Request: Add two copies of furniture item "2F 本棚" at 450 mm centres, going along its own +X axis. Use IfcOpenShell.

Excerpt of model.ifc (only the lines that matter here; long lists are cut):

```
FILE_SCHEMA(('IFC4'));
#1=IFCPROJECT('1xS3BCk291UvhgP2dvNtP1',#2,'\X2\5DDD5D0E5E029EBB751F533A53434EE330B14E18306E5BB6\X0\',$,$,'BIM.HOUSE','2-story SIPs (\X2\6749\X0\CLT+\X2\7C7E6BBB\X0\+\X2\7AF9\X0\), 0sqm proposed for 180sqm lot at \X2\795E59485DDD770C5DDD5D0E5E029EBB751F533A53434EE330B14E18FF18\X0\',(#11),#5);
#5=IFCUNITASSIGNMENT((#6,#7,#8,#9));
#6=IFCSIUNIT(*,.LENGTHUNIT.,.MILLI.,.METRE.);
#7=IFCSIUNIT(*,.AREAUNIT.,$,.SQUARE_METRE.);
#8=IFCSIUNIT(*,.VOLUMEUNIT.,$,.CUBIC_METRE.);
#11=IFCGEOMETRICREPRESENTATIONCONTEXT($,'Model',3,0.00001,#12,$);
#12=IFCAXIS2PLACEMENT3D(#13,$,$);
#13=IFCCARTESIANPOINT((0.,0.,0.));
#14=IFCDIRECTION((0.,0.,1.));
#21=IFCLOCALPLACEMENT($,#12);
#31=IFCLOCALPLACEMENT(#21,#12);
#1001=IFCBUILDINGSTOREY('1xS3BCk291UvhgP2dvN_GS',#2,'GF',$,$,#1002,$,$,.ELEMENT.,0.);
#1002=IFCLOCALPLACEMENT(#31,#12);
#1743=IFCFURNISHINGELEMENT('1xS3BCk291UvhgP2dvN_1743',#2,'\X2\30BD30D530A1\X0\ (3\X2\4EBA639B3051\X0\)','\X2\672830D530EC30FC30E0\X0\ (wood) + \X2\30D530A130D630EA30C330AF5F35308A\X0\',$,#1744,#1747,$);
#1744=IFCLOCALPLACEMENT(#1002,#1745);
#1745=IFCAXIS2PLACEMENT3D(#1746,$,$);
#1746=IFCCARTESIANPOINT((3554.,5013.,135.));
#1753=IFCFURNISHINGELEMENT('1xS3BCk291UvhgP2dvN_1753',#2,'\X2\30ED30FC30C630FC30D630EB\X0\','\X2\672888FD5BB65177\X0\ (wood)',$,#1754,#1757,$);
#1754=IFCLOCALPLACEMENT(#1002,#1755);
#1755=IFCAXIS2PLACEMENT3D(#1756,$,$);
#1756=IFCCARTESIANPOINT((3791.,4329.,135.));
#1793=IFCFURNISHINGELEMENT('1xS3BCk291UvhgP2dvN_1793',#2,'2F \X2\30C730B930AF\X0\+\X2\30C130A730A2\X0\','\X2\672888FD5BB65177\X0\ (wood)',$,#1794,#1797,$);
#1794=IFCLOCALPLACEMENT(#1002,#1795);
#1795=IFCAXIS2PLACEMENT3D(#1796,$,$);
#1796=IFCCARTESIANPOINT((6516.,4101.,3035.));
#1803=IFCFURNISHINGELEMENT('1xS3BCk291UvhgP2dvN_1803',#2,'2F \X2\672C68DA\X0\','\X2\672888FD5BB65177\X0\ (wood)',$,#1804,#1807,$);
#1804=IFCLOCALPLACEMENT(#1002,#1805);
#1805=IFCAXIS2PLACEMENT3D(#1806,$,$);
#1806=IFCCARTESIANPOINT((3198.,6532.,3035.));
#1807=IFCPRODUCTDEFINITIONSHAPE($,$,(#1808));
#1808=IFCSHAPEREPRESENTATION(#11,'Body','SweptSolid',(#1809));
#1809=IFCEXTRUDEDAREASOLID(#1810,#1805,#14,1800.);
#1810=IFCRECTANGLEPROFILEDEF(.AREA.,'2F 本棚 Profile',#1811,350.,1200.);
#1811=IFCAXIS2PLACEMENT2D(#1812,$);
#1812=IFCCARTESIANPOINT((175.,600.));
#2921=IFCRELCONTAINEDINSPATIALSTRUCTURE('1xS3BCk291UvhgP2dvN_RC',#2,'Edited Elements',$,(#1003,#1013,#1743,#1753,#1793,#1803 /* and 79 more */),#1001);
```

```python
import ifcopenshell
import ifcopenshell.api.geometry
import ifcopenshell.api.root
import ifcopenshell.util.element
import ifcopenshell.util.placement
import ifcopenshell.util.unit

model = ifcopenshell.open("model.ifc")
unit_scale = ifcopenshell.util.unit.calculate_unit_scale(model)


def reuse_history(source, copy):
    """copy_class also copies each property set's owner history, people and application; keep the originals."""
    for rel in copy.IsDefinedBy:
        if rel.is_a("IfcRelDefinesByProperties") and (history := rel.RelatingPropertyDefinition.OwnerHistory):
            rel.RelatingPropertyDefinition.OwnerHistory = source.OwnerHistory
            ifcopenshell.util.element.remove_deep2(model, history)


source = model.by_guid("1xS3BCk291UvhgP2dvN_1803")
base = ifcopenshell.util.placement.get_local_placement(source.ObjectPlacement)
step = base[:3, 0] * 0.45 / unit_scale

for i in range(1, 3):
    copy = ifcopenshell.api.root.copy_class(model, product=source)
    copy.Representation = ifcopenshell.util.element.copy_deep(
        model, source.Representation, exclude=["IfcGeometricRepresentationContext", "IfcRepresentationMap"]
    )
    reuse_history(source, copy)
    matrix = base.copy()
    matrix[:3, 3] += i * step
    print("added at", matrix[:3, 3].round(3) + 0.0)
    ifcopenshell.api.geometry.edit_object_placement(model, product=copy, matrix=matrix, is_si=False)

model.write("model_updated.ifc")
```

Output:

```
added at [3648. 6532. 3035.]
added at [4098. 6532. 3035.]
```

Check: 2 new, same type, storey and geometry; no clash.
